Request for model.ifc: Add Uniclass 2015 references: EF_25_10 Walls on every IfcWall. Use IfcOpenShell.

First a look at what the model holds.

```python
import ifcopenshell

model = ifcopenshell.open("model.ifc")
print(model.schema)
print("classifications:", [c.Name for c in model.by_type("IfcClassification")])
for ifc_class in ("IfcDoor", "IfcRoof", "IfcStair", "IfcWall", "IfcWindow"):
    print(ifc_class, len(model.by_type(ifc_class)))
```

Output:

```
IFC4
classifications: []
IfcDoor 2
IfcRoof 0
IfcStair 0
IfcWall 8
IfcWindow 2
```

```python
import ifcopenshell
import ifcopenshell.api.classification

model = ifcopenshell.open("model.ifc")

system = ifcopenshell.api.classification.add_classification(model, classification="Uniclass 2015")

codes = {
    "IfcWall": ("EF_25_10", "Walls"),
}
for ifc_class, (code, name) in codes.items():
    products = model.by_type(ifc_class)
    ifcopenshell.api.classification.add_reference(
        model, products=products, classification=system, identification=code, name=name
    )
    print(code, len(products))

model.write("model-out.ifc")
```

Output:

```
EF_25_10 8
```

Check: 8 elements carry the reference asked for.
